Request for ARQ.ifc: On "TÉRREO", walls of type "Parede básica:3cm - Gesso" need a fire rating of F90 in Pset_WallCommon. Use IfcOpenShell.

First a look at what the model holds.

```python
import ifcopenshell
import ifcopenshell.util.element

model = ifcopenshell.open("ARQ.ifc")
print(model.schema)
storey = next(s for s in model.by_type("IfcBuildingStorey") if s.Name == "TÉRREO")
walls = [e for e in ifcopenshell.util.element.get_decomposition(storey) if e.is_a("IfcWall")]
seen = {}
for e in walls:
    element_type = ifcopenshell.util.element.get_type(e)
    key = (element_type.Name if element_type != e and element_type else None, ifcopenshell.util.element.get_pset(e, "Pset_WallCommon", "FireRating"))
    seen[key] = seen.get(key, 0) + 1
for (name, value), count in sorted(seen.items(), key=str):
    print(count, "x", name, "|", value)
```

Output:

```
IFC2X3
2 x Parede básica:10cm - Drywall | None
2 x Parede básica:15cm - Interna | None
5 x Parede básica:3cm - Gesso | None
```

```python
import ifcopenshell
import ifcopenshell.api.pset
import ifcopenshell.util.element

model = ifcopenshell.open("ARQ.ifc")

storey = next(s for s in model.by_type("IfcBuildingStorey") if s.Name == "TÉRREO")
walls = [e for e in ifcopenshell.util.element.get_decomposition(storey) if e.is_a("IfcWall")]

count = 0
for e in walls:
    element_type = ifcopenshell.util.element.get_type(e)
    if element_type in (None, e) or element_type.Name != "Parede básica:3cm - Gesso":
        continue
    # add_pset returns the element's existing set when there is one.
    pset = ifcopenshell.api.pset.add_pset(model, product=e, name="Pset_WallCommon")
    ifcopenshell.api.pset.edit_pset(model, pset=pset, properties={"FireRating": "F90"})
    count += 1

print(count, "walls updated")

model.write("ARQ_updated.ifc")
```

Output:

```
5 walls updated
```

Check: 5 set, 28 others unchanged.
